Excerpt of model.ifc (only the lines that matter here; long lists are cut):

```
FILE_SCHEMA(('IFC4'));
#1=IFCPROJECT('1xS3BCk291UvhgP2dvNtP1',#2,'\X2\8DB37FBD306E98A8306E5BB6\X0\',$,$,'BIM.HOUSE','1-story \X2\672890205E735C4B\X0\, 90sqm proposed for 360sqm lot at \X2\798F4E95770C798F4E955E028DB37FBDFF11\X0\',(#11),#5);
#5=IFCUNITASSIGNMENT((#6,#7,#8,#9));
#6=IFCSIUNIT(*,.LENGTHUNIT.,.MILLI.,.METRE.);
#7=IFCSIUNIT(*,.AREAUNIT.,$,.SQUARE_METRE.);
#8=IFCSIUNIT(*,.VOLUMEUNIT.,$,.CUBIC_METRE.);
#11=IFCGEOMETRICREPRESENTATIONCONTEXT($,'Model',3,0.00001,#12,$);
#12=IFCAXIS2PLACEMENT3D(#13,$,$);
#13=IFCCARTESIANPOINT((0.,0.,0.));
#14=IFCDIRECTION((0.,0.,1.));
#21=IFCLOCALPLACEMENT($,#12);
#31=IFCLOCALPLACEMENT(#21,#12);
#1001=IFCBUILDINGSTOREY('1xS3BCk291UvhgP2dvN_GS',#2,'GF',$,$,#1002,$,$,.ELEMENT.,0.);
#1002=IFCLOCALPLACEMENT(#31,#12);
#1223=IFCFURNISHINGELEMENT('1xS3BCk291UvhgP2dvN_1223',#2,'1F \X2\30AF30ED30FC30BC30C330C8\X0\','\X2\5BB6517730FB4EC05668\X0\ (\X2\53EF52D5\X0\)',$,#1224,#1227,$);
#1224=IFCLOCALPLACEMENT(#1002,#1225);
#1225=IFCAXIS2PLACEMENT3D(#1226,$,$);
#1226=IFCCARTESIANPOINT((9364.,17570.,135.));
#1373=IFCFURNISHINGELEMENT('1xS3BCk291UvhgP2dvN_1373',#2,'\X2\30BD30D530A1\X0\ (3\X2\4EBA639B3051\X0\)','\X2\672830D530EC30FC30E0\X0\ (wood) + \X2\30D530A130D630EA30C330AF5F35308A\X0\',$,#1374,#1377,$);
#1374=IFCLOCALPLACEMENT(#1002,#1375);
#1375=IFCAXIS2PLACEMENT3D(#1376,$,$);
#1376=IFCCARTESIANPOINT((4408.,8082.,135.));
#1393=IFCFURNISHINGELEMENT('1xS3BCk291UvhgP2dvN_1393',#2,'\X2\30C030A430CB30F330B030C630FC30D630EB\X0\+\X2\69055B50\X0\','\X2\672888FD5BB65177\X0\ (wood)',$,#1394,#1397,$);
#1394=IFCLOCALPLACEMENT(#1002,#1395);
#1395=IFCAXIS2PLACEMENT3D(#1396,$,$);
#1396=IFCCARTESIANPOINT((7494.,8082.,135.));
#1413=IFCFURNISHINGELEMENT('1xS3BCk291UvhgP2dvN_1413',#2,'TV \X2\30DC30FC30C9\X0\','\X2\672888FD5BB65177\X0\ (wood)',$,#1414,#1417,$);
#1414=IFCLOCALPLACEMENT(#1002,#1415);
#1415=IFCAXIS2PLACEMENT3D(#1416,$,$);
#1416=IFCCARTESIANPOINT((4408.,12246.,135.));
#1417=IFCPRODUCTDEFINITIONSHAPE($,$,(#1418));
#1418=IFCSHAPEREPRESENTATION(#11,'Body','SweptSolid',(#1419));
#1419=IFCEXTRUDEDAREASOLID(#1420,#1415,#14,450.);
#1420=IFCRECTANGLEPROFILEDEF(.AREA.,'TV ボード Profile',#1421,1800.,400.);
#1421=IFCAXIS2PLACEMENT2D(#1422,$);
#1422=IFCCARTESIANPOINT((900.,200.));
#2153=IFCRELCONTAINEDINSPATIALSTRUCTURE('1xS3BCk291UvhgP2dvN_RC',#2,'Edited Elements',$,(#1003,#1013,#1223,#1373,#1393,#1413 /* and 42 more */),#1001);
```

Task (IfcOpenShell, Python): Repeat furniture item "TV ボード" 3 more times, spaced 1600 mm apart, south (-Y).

```python
import numpy as np
import ifcopenshell
import ifcopenshell.api.geometry
import ifcopenshell.api.root
import ifcopenshell.util.element
import ifcopenshell.util.placement

model = ifcopenshell.open("model.ifc")


def reuse_history(source, copy):
    """copy_class also copies each property set's owner history, people and application; keep the originals."""
    for rel in copy.IsDefinedBy:
        if rel.is_a("IfcRelDefinesByProperties") and (history := rel.RelatingPropertyDefinition.OwnerHistory):
            rel.RelatingPropertyDefinition.OwnerHistory = source.OwnerHistory
            ifcopenshell.util.element.remove_deep2(model, history)


source = model.by_id(1413)
base = ifcopenshell.util.placement.get_local_placement(source.ObjectPlacement)
step = np.array([0.0, -1.0, 0.0]) * 1600.0

for i in range(1, 4):
    copy = ifcopenshell.api.root.copy_class(model, product=source)
    copy.Representation = ifcopenshell.util.element.copy_deep(
        model, source.Representation, exclude=["IfcGeometricRepresentationContext", "IfcRepresentationMap"]
    )
    reuse_history(source, copy)
    matrix = base.copy()
    matrix[:3, 3] += i * step
    print("added at", matrix[:3, 3].round(3) + 0.0)
    ifcopenshell.api.geometry.edit_object_placement(model, product=copy, matrix=matrix, is_si=False)

model.write("model_updated.ifc")
```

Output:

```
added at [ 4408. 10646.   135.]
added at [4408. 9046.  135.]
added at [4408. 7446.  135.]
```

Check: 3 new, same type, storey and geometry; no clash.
